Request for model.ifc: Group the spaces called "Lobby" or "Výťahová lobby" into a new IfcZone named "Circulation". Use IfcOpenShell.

First a look at what the model holds.

```python
import ifcopenshell

model = ifcopenshell.open("model.ifc")
print(model.schema)
seen = {}
for space in model.by_type("IfcSpace"):
    seen[space.LongName] = seen.get(space.LongName, 0) + 1
for name, count in sorted(seen.items(), key=str):
    print(count, "x", name)
print("zones:", [z.Name for z in model.by_type("IfcZone")][:20])
```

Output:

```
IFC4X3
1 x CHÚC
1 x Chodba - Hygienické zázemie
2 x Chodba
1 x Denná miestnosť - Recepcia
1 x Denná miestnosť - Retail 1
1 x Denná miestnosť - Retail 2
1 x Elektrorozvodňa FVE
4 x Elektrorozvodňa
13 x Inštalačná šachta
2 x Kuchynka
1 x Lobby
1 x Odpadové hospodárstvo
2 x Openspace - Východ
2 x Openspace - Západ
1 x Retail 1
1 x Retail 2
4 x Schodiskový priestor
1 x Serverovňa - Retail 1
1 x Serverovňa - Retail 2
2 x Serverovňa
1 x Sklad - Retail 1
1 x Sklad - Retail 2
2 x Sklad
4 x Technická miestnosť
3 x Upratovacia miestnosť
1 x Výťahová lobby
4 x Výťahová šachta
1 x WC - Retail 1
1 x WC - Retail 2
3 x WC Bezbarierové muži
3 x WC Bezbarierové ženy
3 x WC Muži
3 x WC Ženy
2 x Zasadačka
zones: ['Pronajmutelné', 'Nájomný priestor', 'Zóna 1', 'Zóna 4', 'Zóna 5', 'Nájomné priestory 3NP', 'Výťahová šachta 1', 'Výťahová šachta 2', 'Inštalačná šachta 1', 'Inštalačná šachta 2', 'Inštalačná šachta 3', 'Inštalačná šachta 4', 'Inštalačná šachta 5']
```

```python
import ifcopenshell
import ifcopenshell.api.group
import ifcopenshell.api.root

model = ifcopenshell.open("model.ifc")

names = {"Lobby", "Výťahová lobby"}
spaces = [s for s in model.by_type("IfcSpace") if s.LongName in names]

zone = ifcopenshell.api.root.create_entity(model, ifc_class="IfcZone", name="Circulation")
ifcopenshell.api.group.assign_group(model, products=spaces, group=zone)
print(len(spaces), "spaces in", zone.Name)

model.write("model_v2.ifc")
```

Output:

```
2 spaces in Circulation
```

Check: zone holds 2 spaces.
